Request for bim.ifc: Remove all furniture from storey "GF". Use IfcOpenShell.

First a look at what the model holds.

```python
import ifcopenshell
import ifcopenshell.util.element

model = ifcopenshell.open("bim.ifc")
print(model.schema)
storey = next(s for s in model.by_type("IfcBuildingStorey") if s.Name == "GF")
furniture = [e for e in ifcopenshell.util.element.get_decomposition(storey) if e.is_a("IfcFurnishingElement")]
seen = {}
for e in furniture:
    element_type = ifcopenshell.util.element.get_type(e)
    name = element_type.Name if element_type not in (None, e) else None
    seen[name] = seen.get(name, 0) + 1
for name, count in sorted(seen.items(), key=str):
    print(count, "x", name)
```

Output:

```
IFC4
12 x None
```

```python
import ifcopenshell
import ifcopenshell.api.root
import ifcopenshell.util.element

model = ifcopenshell.open("bim.ifc")

storey = next(s for s in model.by_type("IfcBuildingStorey") if s.Name == "GF")
furniture = [e for e in ifcopenshell.util.element.get_decomposition(storey) if e.is_a("IfcFurnishingElement")]

for e in furniture:
    ifcopenshell.api.root.remove_product(model, product=e)
print(len(furniture), "removed")

model.write("bim_edited.ifc")
```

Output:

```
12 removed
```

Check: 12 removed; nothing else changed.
